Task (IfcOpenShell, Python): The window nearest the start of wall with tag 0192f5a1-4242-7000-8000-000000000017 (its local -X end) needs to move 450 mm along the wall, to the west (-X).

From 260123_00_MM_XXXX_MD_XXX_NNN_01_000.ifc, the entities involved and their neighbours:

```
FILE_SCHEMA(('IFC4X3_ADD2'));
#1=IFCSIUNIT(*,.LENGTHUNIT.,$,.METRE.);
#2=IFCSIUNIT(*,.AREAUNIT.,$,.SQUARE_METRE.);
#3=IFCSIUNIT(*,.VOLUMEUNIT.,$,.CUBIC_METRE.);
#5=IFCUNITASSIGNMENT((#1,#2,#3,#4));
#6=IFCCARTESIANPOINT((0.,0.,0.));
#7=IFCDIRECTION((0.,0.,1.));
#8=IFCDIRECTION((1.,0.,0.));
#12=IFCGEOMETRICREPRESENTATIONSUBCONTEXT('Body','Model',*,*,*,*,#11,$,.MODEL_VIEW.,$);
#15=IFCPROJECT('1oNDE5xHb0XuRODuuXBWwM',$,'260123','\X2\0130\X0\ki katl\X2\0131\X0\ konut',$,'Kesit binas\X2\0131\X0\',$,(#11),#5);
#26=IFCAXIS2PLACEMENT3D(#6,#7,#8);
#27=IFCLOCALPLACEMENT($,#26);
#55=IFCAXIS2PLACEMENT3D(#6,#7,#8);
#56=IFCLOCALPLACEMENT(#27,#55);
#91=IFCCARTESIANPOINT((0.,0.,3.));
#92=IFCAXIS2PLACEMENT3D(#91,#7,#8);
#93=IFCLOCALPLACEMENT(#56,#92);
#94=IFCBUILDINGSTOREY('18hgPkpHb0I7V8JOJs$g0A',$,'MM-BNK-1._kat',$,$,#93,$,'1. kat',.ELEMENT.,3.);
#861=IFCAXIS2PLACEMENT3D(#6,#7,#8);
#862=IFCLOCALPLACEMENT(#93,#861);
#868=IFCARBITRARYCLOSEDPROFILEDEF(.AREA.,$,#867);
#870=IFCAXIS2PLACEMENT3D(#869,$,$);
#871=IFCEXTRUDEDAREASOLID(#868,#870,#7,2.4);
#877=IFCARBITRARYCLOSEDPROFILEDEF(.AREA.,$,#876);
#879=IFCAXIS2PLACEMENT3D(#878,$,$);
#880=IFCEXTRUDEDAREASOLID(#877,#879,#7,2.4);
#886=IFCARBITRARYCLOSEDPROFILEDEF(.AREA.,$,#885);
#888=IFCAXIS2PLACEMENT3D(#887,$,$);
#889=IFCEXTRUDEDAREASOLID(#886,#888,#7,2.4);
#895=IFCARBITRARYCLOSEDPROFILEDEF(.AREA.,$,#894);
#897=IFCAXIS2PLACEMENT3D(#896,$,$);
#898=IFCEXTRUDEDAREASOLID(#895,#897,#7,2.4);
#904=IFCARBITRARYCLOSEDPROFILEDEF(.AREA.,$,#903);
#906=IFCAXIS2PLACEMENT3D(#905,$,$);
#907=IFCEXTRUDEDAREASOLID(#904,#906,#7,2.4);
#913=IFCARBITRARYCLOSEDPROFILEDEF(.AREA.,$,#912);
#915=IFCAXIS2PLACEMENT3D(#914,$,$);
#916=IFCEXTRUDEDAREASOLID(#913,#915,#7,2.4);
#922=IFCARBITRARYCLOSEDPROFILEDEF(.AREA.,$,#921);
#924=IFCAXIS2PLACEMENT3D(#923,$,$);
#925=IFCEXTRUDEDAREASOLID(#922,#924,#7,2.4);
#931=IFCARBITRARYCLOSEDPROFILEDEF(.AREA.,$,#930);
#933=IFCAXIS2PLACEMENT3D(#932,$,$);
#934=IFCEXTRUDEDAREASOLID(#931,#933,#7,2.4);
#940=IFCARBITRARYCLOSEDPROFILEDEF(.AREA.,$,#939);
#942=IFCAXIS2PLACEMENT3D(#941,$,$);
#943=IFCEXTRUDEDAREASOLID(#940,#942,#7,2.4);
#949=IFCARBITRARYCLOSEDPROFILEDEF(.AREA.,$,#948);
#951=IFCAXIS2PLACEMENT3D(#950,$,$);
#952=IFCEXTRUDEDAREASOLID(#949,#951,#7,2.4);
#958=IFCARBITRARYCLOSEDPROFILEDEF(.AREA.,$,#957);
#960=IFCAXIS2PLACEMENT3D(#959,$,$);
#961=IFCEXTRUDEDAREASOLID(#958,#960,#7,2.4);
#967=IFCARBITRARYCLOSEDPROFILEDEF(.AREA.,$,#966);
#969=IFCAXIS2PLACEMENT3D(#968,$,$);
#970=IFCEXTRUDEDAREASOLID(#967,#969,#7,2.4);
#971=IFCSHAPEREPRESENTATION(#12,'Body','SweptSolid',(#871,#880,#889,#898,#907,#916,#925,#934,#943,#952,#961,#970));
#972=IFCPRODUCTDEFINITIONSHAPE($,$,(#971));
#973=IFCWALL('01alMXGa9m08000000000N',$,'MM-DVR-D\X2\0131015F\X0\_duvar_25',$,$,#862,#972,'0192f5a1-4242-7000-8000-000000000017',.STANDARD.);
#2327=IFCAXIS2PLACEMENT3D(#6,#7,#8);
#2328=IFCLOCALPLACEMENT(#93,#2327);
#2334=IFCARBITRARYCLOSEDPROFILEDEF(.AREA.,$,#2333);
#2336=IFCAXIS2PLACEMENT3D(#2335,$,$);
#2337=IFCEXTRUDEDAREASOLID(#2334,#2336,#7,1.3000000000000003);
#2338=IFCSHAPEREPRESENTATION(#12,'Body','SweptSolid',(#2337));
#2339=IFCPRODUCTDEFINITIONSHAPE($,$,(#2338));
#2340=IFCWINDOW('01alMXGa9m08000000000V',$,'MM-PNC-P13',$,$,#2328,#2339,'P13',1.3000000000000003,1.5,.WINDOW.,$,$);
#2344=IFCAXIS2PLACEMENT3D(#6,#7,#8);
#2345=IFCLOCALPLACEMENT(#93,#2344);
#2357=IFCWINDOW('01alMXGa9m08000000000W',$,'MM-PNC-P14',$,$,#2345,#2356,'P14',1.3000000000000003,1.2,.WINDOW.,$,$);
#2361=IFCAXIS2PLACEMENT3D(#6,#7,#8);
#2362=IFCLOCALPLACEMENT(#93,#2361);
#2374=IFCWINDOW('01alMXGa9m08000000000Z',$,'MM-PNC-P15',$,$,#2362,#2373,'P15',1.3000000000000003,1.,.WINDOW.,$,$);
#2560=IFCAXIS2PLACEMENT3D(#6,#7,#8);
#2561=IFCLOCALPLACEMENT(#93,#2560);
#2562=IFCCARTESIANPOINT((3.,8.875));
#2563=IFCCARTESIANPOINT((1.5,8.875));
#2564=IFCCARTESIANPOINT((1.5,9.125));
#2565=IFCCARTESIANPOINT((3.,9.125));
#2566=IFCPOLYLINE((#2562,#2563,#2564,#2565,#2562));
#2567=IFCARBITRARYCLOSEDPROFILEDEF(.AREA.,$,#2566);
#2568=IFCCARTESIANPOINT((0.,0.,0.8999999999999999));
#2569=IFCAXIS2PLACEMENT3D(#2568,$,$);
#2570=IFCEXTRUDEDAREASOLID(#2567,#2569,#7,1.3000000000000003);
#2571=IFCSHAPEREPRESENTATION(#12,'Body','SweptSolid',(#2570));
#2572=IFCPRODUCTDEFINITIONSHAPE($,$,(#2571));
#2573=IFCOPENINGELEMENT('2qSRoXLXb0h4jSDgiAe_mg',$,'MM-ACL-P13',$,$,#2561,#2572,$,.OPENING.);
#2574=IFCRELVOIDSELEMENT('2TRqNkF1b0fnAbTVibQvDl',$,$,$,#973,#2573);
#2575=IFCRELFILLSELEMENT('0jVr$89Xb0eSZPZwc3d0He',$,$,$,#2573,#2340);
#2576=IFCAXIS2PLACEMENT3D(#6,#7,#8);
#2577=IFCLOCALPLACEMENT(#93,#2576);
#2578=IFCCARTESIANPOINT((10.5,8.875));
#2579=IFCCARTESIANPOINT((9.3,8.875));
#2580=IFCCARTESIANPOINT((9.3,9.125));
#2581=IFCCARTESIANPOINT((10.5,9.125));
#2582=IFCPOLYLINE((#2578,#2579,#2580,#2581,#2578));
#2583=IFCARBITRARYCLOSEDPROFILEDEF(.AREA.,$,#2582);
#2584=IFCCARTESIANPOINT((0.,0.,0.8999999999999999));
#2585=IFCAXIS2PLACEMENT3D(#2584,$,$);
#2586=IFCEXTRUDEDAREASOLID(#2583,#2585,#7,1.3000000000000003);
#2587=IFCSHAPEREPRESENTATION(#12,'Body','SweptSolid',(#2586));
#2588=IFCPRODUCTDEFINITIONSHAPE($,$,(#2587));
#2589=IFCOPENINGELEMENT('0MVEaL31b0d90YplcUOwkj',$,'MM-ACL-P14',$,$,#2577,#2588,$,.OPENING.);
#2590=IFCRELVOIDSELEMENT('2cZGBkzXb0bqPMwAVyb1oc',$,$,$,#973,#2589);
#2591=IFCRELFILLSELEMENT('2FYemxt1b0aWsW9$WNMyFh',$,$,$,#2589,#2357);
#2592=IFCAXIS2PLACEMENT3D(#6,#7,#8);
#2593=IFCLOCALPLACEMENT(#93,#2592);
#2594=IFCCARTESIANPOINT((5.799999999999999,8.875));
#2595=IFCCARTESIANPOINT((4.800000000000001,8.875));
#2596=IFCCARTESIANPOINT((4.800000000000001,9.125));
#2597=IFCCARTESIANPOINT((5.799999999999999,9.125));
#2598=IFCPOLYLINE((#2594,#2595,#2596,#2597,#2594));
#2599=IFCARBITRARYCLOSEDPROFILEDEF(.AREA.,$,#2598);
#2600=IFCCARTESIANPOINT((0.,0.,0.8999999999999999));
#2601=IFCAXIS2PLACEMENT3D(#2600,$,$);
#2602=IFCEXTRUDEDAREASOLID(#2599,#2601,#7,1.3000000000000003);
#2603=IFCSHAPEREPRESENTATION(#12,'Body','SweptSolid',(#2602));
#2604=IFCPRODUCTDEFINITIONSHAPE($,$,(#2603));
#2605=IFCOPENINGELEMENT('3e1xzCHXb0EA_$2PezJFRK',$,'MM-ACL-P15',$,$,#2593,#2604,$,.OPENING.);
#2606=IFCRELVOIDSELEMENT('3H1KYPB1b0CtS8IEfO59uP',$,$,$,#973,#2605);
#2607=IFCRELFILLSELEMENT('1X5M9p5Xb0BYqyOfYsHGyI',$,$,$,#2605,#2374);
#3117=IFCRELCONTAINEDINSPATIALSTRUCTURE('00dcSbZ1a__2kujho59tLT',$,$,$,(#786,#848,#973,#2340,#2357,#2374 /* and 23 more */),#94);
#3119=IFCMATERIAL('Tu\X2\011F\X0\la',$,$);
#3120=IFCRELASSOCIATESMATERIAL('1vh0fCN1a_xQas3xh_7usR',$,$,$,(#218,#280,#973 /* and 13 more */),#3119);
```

```python
import ifcopenshell
import ifcopenshell.api.geometry
import ifcopenshell.util.placement
import ifcopenshell.util.unit

model = ifcopenshell.open("260123_00_MM_XXXX_MD_XXX_NNN_01_000.ifc")
unit_scale = ifcopenshell.util.unit.calculate_unit_scale(model)

window = model.by_guid("01alMXGa9m08000000000V")
opening = window.FillsVoids[0].RelatingOpeningElement
wall = opening.VoidsElements[0].RelatingBuildingElement

wall_matrix = ifcopenshell.util.placement.get_local_placement(wall.ObjectPlacement)
shift = wall_matrix[:3, 0] * -0.45 / unit_scale
before = ifcopenshell.util.placement.get_local_placement(window.ObjectPlacement)[:3, 3].copy()

# The window is not placed relative to its opening, so move both.
for product in (opening, window):
    matrix = ifcopenshell.util.placement.get_local_placement(product.ObjectPlacement)
    matrix[:3, 3] += shift
    ifcopenshell.api.geometry.edit_object_placement(model, product=product, matrix=matrix, is_si=False)

after = ifcopenshell.util.placement.get_local_placement(window.ObjectPlacement)[:3, 3]
print("window moved by", (after - before).round(3) + 0.0)

model.write("260123_00_MM_XXXX_MD_XXX_NNN_01_000_v2.ifc")
```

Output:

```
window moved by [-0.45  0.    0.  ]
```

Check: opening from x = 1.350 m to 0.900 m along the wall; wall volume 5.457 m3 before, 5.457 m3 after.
